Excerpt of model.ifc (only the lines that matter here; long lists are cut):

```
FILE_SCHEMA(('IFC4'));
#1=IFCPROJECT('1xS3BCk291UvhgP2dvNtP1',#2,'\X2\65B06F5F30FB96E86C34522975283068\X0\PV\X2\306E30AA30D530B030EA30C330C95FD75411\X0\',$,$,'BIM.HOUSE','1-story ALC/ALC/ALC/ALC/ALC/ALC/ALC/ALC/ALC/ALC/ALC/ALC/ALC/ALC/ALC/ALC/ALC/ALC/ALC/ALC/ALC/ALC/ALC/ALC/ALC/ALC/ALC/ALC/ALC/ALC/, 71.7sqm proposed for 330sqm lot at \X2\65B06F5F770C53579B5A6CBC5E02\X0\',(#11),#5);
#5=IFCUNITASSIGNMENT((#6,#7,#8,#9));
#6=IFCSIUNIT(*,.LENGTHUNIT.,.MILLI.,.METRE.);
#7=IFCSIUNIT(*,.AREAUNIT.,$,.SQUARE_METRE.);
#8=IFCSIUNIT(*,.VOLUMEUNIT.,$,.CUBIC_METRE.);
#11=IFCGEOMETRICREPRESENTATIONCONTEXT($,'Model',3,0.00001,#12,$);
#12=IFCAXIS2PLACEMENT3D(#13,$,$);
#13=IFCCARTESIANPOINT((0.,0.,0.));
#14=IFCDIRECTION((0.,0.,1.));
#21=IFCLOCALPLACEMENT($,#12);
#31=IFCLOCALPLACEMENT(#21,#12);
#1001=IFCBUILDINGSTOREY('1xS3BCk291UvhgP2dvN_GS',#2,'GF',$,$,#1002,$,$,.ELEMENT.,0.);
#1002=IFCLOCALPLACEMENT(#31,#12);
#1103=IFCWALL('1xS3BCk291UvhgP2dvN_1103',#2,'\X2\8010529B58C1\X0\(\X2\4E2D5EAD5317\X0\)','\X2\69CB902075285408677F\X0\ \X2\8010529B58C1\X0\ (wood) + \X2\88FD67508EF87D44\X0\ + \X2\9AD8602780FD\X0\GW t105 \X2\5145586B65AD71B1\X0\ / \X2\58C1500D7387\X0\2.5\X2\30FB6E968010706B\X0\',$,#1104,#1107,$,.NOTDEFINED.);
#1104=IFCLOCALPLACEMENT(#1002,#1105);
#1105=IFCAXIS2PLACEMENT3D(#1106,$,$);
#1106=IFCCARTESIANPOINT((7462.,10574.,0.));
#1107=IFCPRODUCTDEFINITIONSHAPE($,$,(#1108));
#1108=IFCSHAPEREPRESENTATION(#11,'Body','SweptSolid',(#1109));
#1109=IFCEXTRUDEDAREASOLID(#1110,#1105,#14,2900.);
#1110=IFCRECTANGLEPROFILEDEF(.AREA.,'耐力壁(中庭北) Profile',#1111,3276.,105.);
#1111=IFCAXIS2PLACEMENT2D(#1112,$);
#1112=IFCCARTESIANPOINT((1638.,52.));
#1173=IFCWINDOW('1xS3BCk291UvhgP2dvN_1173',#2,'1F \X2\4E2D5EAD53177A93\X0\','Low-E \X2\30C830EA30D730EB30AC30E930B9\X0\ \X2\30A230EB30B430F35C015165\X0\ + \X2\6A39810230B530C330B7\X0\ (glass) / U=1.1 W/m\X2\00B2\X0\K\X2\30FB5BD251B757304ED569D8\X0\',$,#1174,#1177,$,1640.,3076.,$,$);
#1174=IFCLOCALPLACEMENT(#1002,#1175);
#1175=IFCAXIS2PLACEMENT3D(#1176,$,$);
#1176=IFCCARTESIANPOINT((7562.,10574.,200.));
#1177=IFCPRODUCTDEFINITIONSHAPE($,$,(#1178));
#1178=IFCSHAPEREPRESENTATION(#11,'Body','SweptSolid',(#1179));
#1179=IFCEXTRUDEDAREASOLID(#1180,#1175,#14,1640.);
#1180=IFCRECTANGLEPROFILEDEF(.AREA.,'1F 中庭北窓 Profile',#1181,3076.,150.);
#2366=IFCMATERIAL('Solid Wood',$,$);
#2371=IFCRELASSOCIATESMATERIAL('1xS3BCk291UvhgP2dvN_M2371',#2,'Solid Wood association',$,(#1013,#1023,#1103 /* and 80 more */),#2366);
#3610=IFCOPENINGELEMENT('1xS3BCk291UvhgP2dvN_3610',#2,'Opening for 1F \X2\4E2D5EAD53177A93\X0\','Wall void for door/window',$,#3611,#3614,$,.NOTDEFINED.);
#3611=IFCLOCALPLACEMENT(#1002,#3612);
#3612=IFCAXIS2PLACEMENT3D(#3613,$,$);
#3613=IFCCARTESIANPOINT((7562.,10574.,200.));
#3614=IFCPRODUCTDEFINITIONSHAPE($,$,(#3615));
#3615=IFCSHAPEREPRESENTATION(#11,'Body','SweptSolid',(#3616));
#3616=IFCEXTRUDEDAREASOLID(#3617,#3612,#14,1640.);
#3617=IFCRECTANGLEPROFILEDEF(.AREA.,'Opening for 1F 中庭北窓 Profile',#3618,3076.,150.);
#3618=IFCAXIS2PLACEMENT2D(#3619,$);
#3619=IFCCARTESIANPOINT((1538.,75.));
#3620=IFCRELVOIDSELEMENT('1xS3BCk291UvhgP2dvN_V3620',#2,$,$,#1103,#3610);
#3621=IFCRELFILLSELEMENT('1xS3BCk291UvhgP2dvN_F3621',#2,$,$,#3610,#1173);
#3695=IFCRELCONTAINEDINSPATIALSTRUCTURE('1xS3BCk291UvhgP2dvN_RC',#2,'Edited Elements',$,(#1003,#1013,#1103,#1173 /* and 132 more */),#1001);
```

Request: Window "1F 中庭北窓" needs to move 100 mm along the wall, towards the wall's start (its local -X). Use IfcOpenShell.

```python
import ifcopenshell
import ifcopenshell.api.geometry
import ifcopenshell.util.placement
import ifcopenshell.util.unit

model = ifcopenshell.open("model.ifc")
unit_scale = ifcopenshell.util.unit.calculate_unit_scale(model)

window = model.by_guid("1xS3BCk291UvhgP2dvN_1173")
opening = window.FillsVoids[0].RelatingOpeningElement
wall = opening.VoidsElements[0].RelatingBuildingElement

wall_matrix = ifcopenshell.util.placement.get_local_placement(wall.ObjectPlacement)
shift = wall_matrix[:3, 0] * -0.1 / unit_scale
before = ifcopenshell.util.placement.get_local_placement(window.ObjectPlacement)[:3, 3].copy()

# The window is not placed relative to its opening, so move both.
for product in (opening, window):
    matrix = ifcopenshell.util.placement.get_local_placement(product.ObjectPlacement)
    matrix[:3, 3] += shift
    ifcopenshell.api.geometry.edit_object_placement(model, product=product, matrix=matrix, is_si=False)

after = ifcopenshell.util.placement.get_local_placement(window.ObjectPlacement)[:3, 3]
print("window moved by", (after - before).round(3) + 0.0)

model.write("model_edited.ifc")
```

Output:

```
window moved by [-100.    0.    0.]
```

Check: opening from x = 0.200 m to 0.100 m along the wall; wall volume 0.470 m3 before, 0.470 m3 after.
